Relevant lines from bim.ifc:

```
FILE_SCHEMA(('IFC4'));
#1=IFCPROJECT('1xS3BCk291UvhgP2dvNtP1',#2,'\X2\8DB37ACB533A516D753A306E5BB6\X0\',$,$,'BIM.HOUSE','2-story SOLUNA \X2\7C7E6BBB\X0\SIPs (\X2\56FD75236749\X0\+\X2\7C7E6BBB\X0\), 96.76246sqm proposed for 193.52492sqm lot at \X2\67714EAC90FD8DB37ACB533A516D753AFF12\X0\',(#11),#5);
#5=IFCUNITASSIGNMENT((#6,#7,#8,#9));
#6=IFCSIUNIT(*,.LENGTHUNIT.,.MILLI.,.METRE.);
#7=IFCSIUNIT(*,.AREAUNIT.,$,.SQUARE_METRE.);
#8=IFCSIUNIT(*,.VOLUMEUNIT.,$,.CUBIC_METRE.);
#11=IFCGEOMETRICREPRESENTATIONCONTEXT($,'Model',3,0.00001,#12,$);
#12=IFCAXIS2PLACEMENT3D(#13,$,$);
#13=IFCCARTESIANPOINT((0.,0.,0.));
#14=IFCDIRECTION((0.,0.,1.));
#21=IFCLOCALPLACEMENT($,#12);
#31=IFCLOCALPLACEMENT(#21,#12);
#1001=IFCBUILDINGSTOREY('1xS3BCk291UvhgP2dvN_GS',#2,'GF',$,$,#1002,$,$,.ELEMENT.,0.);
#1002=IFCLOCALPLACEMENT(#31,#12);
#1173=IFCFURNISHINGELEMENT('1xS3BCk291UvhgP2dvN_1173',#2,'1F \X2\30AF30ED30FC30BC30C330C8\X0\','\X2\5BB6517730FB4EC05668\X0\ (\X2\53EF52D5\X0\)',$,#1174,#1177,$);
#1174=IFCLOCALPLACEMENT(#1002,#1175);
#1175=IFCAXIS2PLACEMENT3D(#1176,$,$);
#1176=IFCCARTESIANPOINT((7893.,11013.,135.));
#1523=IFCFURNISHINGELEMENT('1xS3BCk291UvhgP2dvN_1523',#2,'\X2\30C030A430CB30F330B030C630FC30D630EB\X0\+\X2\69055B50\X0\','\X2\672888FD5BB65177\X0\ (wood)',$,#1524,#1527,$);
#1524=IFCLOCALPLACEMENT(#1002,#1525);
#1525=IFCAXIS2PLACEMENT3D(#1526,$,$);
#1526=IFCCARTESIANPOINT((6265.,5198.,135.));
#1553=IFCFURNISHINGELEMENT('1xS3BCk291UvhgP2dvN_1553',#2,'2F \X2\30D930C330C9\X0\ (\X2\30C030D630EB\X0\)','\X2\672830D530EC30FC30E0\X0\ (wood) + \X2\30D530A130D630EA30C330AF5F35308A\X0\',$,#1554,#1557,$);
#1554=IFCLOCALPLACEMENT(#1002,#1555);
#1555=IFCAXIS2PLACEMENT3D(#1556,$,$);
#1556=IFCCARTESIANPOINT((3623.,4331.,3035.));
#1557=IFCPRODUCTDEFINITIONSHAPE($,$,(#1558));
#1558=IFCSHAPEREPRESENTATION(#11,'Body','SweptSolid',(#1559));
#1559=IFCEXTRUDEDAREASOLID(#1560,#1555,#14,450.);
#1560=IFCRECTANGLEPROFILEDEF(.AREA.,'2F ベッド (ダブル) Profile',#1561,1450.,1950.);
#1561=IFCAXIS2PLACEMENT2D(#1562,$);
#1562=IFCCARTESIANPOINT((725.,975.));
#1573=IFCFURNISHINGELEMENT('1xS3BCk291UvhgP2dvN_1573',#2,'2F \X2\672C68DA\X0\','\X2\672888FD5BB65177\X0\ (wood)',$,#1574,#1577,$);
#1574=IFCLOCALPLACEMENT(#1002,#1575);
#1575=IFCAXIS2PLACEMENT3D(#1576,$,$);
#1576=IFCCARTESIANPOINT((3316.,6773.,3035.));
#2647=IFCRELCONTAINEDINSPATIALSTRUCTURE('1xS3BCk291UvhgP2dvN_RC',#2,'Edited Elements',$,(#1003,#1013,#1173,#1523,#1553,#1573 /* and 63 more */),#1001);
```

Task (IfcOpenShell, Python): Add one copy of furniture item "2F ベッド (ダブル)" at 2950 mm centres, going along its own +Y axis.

```python
import ifcopenshell
import ifcopenshell.api.geometry
import ifcopenshell.api.root
import ifcopenshell.util.element
import ifcopenshell.util.placement
import ifcopenshell.util.unit

model = ifcopenshell.open("bim.ifc")
unit_scale = ifcopenshell.util.unit.calculate_unit_scale(model)


def reuse_history(source, copy):
    """copy_class also copies each property set's owner history, people and application; keep the originals."""
    for rel in copy.IsDefinedBy:
        if rel.is_a("IfcRelDefinesByProperties") and (history := rel.RelatingPropertyDefinition.OwnerHistory):
            rel.RelatingPropertyDefinition.OwnerHistory = source.OwnerHistory
            ifcopenshell.util.element.remove_deep2(model, history)


source = model.by_guid("1xS3BCk291UvhgP2dvN_1553")
base = ifcopenshell.util.placement.get_local_placement(source.ObjectPlacement)
step = base[:3, 1] * 2.95 / unit_scale

for i in range(1, 2):
    copy = ifcopenshell.api.root.copy_class(model, product=source)
    copy.Representation = ifcopenshell.util.element.copy_deep(
        model, source.Representation, exclude=["IfcGeometricRepresentationContext", "IfcRepresentationMap"]
    )
    reuse_history(source, copy)
    matrix = base.copy()
    matrix[:3, 3] += i * step
    print("added at", matrix[:3, 3].round(3) + 0.0)
    ifcopenshell.api.geometry.edit_object_placement(model, product=copy, matrix=matrix, is_si=False)

model.write("bim_edited.ifc")
```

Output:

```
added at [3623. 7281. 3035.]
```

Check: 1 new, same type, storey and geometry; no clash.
